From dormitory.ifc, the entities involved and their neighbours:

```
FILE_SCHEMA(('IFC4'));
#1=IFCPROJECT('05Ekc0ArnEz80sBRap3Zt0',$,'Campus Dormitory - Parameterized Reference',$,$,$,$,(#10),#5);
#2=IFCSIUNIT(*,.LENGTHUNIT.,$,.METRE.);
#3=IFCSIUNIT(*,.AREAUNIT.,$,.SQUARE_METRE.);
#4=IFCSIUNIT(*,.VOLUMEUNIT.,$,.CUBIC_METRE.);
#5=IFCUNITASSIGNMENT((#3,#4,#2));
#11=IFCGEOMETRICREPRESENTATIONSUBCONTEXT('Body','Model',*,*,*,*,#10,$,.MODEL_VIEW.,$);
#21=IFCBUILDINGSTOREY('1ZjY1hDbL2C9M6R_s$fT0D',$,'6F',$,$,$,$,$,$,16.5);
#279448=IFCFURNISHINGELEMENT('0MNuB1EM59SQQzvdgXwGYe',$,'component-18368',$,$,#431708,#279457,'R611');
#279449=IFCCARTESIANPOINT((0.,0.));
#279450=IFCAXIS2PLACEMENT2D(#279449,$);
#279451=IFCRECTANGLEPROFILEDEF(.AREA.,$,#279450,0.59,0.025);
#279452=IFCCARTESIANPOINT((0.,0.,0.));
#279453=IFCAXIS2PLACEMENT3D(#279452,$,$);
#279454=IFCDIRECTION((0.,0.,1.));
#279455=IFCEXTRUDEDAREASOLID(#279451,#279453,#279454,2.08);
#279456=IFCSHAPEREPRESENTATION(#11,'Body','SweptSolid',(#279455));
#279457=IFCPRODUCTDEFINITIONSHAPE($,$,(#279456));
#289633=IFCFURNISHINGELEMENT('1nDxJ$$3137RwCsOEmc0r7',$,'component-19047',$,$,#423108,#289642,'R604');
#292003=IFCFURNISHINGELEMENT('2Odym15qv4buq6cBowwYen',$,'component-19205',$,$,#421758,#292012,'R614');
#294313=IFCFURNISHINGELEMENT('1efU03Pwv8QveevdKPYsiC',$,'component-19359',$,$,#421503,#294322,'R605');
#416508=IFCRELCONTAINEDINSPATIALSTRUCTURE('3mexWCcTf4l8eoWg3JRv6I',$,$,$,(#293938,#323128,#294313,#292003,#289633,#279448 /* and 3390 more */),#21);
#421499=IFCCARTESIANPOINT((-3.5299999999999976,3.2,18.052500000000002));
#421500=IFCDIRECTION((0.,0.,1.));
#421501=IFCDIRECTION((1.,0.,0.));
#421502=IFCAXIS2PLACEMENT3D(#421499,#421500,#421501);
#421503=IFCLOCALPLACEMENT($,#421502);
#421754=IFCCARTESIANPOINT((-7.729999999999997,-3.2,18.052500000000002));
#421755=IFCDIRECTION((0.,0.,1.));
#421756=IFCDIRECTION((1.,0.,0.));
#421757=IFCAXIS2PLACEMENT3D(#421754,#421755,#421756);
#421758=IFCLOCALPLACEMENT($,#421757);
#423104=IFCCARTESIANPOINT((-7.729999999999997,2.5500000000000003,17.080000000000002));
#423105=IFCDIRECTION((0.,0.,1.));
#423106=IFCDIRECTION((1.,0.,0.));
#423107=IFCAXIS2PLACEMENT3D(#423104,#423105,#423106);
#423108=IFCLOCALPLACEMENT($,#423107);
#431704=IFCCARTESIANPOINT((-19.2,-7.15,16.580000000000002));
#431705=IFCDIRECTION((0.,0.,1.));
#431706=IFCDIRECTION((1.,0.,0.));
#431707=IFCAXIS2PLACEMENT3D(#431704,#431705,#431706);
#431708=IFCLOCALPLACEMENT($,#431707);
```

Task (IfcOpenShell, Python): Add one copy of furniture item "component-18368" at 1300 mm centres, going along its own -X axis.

```python
import ifcopenshell
import ifcopenshell.api.geometry
import ifcopenshell.api.root
import ifcopenshell.util.element
import ifcopenshell.util.placement
import ifcopenshell.util.unit

model = ifcopenshell.open("dormitory.ifc")
unit_scale = ifcopenshell.util.unit.calculate_unit_scale(model)

source = model.by_guid("0MNuB1EM59SQQzvdgXwGYe")
base = ifcopenshell.util.placement.get_local_placement(source.ObjectPlacement)
step = -base[:3, 0] * 1.3 / unit_scale

for i in range(1, 2):
    copy = ifcopenshell.api.root.copy_class(model, product=source)
    copy.Representation = ifcopenshell.util.element.copy_deep(
        model, source.Representation, exclude=["IfcGeometricRepresentationContext", "IfcRepresentationMap"]
    )
    copy.Tag = None
    matrix = base.copy()
    matrix[:3, 3] += i * step
    print("added at", matrix[:3, 3].round(3) + 0.0)
    ifcopenshell.api.geometry.edit_object_placement(model, product=copy, matrix=matrix, is_si=False)

model.write("dormitory_v2.ifc")
```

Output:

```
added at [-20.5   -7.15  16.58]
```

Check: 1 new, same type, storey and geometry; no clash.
